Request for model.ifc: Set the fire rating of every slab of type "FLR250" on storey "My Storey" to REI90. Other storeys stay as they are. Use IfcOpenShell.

First a look at what the model holds.

```python
import ifcopenshell
import ifcopenshell.util.element

model = ifcopenshell.open("model.ifc")
print(model.schema)
storey = next(s for s in model.by_type("IfcBuildingStorey") if s.Name == "My Storey")
slabs = [e for e in ifcopenshell.util.element.get_decomposition(storey) if e.is_a("IfcSlab")]
seen = {}
for e in slabs:
    element_type = ifcopenshell.util.element.get_type(e)
    key = (element_type.Name if element_type != e and element_type else None, ifcopenshell.util.element.get_pset(e, "Pset_SlabCommon", "FireRating"))
    seen[key] = seen.get(key, 0) + 1
for (name, value), count in sorted(seen.items(), key=str):
    print(count, "x", name, "|", value)
```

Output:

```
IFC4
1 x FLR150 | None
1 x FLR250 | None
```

```python
import ifcopenshell
import ifcopenshell.api.pset
import ifcopenshell.util.element

model = ifcopenshell.open("model.ifc")

storey = next(s for s in model.by_type("IfcBuildingStorey") if s.Name == "My Storey")
slabs = [e for e in ifcopenshell.util.element.get_decomposition(storey) if e.is_a("IfcSlab")]

count = 0
for e in slabs:
    element_type = ifcopenshell.util.element.get_type(e)
    if element_type in (None, e) or element_type.Name != "FLR250":
        continue
    # add_pset returns the element's existing set when there is one.
    pset = ifcopenshell.api.pset.add_pset(model, product=e, name="Pset_SlabCommon")
    ifcopenshell.api.pset.edit_pset(model, pset=pset, properties={"FireRating": "REI90"})
    count += 1

print(count, "slabs updated")

model.write("model-out.ifc")
```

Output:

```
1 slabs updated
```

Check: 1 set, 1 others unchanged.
